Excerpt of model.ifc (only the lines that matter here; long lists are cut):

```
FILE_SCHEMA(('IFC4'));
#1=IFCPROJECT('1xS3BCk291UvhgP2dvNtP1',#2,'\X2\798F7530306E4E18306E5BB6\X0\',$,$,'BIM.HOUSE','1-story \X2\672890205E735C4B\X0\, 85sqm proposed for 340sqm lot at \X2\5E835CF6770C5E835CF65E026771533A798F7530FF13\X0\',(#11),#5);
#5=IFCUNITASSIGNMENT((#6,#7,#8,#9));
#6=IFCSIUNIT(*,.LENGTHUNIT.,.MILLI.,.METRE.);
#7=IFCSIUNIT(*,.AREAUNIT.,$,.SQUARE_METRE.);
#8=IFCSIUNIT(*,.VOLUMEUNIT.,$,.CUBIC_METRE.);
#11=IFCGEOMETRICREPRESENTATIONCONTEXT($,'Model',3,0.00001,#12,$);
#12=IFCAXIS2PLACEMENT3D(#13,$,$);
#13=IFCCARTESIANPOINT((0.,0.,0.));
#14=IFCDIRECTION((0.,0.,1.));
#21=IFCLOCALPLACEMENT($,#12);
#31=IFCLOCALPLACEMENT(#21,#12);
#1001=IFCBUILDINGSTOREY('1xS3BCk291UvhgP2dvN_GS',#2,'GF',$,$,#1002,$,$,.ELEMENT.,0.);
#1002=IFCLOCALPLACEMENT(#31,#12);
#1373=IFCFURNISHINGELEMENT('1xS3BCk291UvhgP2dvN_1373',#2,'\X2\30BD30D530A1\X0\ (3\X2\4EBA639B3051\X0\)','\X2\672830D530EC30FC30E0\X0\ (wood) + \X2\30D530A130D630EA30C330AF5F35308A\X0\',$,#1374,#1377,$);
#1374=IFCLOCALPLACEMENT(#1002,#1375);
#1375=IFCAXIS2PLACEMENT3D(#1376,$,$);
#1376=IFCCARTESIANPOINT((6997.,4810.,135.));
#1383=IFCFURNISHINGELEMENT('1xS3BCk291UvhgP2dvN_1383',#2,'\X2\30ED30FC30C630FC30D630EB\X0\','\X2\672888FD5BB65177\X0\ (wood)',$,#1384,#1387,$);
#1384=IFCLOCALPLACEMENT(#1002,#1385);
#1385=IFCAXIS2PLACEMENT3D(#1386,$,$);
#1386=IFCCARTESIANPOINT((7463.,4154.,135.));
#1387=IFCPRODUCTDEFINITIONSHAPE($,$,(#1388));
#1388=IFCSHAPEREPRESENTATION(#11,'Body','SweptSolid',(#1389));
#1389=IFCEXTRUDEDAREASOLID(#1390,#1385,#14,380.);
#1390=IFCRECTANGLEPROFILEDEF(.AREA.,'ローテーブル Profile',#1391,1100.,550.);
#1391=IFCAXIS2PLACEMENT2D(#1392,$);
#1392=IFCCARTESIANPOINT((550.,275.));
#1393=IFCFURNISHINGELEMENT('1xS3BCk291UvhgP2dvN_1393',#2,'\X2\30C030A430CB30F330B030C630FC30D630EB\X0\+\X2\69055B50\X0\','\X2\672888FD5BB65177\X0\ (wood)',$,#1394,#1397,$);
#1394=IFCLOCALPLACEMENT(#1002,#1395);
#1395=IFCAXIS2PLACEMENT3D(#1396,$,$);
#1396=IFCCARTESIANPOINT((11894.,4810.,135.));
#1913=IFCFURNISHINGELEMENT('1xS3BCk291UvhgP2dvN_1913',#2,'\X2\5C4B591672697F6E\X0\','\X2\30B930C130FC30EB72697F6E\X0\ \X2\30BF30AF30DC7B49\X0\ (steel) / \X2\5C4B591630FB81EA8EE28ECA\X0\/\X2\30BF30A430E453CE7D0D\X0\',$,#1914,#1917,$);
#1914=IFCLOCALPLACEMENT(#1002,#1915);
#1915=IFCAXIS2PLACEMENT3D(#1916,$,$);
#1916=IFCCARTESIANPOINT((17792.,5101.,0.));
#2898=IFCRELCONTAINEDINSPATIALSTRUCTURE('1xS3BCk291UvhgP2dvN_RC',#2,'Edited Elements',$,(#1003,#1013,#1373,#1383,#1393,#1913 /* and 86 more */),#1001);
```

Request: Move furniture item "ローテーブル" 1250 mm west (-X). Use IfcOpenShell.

```python
import ifcopenshell
import ifcopenshell.api.geometry
import ifcopenshell.util.placement

model = ifcopenshell.open("model.ifc")

item = model.by_guid("1xS3BCk291UvhgP2dvN_1383")
matrix = ifcopenshell.util.placement.get_local_placement(item.ObjectPlacement)
matrix[0, 3] -= 1250.0
ifcopenshell.api.geometry.edit_object_placement(model, product=item, matrix=matrix, is_si=False)

print(ifcopenshell.util.placement.get_local_placement(item.ObjectPlacement).round(3) + 0.0)

model.write("model_updated.ifc")
```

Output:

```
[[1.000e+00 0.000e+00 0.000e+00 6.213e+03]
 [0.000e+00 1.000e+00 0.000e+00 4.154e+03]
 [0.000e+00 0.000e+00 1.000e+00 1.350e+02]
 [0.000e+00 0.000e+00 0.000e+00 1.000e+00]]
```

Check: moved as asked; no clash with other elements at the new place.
